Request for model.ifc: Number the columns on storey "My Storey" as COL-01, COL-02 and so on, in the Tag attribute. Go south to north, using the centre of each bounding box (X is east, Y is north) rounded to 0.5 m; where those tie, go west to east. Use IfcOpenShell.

First a look at what the model holds.

```python
import ifcopenshell
import ifcopenshell.util.element
import ifcopenshell.util.placement

model = ifcopenshell.open("model.ifc")
print(model.schema)
storey = next(s for s in model.by_type("IfcBuildingStorey") if s.Name == "My Storey")
columns = [e for e in ifcopenshell.util.element.get_decomposition(storey) if e.is_a("IfcColumn")]
for e in sorted(columns, key=lambda e: e.id()):
    origin = ifcopenshell.util.placement.get_local_placement(e.ObjectPlacement)[:3, 3]
    print(e.id(), e.Tag, e.Name, origin.round(2) + 0.0, sep=" | ")
```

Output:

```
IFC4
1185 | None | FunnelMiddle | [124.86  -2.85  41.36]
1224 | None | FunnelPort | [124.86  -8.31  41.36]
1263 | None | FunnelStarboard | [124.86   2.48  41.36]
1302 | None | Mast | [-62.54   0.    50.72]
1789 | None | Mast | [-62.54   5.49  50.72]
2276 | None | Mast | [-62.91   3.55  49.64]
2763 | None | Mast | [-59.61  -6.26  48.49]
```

```python
import ifcopenshell
import ifcopenshell.geom
import ifcopenshell.util.element
import ifcopenshell.util.shape

model = ifcopenshell.open("model.ifc")
settings = ifcopenshell.geom.settings()
settings.set("use-world-coords", True)


def centre(element):
    shape = ifcopenshell.geom.create_shape(settings, element)
    return ifcopenshell.util.shape.get_bbox_centroid(shape.geometry)


storey = next(s for s in model.by_type("IfcBuildingStorey") if s.Name == "My Storey")
columns = [e for e in ifcopenshell.util.element.get_decomposition(storey) if e.is_a("IfcColumn")]

# Insertion points can sit at a corner or the storey origin, so sort by the geometry (in metres).
centres = {e: centre(e) for e in columns}
columns.sort(key=lambda e: (round(centres[e][1] / 0.5), centres[e][0]))

for i, e in enumerate(columns, start=1):
    number = f"COL-{i:02d}"
    e.Tag = number
    print(e.id(), number)

model.write("model-out.ifc")
```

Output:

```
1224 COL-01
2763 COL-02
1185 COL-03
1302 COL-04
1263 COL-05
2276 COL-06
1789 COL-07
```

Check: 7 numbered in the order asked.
